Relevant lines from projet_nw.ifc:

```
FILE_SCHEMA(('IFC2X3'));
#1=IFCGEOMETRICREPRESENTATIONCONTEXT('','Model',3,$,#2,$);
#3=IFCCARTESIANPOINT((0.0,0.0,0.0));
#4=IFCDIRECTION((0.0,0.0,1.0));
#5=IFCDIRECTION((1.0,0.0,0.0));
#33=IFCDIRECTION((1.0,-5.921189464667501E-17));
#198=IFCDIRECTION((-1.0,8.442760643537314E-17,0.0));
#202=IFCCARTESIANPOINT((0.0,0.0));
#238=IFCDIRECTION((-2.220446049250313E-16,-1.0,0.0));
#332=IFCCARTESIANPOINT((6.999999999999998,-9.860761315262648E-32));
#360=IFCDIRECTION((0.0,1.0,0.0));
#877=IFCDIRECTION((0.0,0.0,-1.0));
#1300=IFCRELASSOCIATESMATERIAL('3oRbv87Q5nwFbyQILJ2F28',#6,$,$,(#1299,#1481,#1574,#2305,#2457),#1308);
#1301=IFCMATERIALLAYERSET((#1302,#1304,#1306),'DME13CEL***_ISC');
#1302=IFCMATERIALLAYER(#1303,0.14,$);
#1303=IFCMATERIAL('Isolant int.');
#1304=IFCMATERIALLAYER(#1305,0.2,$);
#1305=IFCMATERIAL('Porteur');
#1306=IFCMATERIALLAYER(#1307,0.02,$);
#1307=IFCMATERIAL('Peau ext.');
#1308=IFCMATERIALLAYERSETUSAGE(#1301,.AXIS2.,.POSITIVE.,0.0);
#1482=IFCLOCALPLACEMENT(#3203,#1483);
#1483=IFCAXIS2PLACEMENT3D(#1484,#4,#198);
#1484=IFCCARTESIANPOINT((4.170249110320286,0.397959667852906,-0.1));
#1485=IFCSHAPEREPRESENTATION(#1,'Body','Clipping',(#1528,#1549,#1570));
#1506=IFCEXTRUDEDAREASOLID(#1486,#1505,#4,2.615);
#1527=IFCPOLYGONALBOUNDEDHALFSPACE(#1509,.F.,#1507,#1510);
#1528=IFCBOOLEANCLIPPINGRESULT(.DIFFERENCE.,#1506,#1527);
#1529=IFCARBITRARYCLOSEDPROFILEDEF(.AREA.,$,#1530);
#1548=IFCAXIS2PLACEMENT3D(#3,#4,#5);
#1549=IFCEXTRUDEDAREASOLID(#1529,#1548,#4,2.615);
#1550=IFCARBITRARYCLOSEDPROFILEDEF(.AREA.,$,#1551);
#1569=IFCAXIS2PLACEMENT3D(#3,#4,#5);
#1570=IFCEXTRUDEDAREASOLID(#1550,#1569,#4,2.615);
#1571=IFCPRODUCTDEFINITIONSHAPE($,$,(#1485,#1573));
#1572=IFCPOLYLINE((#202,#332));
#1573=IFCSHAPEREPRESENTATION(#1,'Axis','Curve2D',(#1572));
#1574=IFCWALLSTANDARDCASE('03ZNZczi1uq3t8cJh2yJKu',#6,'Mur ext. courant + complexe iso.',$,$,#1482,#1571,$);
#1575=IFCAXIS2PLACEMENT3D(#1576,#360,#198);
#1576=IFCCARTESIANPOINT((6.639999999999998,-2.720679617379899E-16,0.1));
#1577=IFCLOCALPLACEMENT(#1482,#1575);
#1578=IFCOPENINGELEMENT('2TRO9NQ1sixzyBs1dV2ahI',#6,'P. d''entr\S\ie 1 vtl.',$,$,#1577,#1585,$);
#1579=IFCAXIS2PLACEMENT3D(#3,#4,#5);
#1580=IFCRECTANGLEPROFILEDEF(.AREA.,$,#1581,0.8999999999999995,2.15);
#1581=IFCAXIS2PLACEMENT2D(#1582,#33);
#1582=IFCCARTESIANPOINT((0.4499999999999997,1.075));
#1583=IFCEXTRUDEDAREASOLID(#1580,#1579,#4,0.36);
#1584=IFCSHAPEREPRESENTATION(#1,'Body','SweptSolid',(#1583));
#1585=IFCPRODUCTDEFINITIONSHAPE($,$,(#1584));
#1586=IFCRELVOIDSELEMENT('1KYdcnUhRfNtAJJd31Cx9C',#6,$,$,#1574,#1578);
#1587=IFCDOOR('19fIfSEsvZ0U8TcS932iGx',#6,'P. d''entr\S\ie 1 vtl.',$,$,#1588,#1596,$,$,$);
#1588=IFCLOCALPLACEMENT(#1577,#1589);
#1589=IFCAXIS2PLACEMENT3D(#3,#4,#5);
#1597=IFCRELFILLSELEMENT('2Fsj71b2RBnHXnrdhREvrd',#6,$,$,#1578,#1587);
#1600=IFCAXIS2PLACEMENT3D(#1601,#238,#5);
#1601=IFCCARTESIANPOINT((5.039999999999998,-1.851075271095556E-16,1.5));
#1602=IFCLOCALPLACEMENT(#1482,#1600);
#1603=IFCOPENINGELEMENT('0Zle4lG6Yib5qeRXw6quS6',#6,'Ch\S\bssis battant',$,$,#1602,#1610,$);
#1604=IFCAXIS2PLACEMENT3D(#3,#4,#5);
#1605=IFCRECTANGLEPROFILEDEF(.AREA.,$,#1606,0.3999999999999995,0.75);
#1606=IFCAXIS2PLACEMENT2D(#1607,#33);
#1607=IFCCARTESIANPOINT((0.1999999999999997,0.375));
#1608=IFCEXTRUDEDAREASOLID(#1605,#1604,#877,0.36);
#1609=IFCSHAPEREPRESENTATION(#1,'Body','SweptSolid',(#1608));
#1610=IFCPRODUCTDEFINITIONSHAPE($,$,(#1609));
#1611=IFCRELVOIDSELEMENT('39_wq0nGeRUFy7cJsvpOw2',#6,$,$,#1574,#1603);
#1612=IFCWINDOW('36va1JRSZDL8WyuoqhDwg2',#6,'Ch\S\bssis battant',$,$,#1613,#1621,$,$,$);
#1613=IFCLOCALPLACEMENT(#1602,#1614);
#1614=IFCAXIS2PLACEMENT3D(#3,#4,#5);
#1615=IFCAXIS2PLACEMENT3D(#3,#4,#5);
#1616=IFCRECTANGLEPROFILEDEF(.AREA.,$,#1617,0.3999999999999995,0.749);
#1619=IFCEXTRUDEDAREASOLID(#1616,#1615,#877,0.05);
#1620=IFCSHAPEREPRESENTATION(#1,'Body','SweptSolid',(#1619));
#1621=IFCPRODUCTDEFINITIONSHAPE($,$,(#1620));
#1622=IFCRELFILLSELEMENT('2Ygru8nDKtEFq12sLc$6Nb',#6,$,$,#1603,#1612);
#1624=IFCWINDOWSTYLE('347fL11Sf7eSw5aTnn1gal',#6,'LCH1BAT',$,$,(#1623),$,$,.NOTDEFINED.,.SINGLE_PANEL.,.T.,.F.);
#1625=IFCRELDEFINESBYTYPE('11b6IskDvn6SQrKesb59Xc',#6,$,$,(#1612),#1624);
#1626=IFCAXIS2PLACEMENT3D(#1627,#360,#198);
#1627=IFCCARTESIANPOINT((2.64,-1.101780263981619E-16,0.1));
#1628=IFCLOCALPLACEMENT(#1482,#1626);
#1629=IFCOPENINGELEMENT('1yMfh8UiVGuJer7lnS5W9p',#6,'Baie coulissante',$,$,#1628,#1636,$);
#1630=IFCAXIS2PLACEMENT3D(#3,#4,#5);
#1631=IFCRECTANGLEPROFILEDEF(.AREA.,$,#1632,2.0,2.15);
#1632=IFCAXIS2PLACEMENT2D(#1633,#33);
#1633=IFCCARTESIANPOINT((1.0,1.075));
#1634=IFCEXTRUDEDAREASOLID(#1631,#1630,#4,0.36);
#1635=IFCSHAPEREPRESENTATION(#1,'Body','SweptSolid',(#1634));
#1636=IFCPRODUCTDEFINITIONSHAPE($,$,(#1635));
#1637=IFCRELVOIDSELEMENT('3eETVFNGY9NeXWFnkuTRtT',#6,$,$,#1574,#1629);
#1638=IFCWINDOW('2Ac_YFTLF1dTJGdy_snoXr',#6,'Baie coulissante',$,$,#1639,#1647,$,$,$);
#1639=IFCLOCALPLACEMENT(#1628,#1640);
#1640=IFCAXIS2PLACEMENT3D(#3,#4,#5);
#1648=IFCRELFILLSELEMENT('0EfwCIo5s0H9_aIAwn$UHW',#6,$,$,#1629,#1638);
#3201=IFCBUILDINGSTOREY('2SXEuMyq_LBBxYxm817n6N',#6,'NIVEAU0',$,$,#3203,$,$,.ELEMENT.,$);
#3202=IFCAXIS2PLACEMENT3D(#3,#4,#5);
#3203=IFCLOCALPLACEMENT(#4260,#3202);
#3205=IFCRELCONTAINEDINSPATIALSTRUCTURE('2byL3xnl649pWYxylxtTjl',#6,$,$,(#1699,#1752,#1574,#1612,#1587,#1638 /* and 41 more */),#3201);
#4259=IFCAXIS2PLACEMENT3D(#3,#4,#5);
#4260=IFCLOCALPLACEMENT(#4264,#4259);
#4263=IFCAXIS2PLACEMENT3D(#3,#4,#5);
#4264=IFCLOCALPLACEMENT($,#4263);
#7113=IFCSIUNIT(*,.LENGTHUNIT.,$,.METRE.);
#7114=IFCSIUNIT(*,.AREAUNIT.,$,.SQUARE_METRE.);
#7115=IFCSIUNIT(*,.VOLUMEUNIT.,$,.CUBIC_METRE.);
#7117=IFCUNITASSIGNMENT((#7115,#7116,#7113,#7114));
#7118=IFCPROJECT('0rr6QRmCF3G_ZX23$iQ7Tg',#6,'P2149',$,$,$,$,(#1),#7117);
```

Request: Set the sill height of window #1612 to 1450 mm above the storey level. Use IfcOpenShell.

```python
import numpy as np
import ifcopenshell
import ifcopenshell.api.geometry
import ifcopenshell.geom
import ifcopenshell.util.element
import ifcopenshell.util.placement
import ifcopenshell.util.shape
import ifcopenshell.util.unit

model = ifcopenshell.open("projet_nw.ifc")
unit_scale = ifcopenshell.util.unit.calculate_unit_scale(model)

window = model.by_guid("36va1JRSZDL8WyuoqhDwg2")
opening = window.FillsVoids[0].RelatingOpeningElement
storey = ifcopenshell.util.element.get_container(window, ifc_class="IfcBuildingStorey")
level = ifcopenshell.util.placement.get_local_placement(storey.ObjectPlacement)[2, 3]

# The opening's origin need not be at the sill, so measure its lowest point.
shape = ifcopenshell.geom.create_shape(ifcopenshell.geom.settings(), opening)
bottom = ifcopenshell.util.shape.get_shape_bottom_elevation(shape, shape.geometry) / unit_scale
dz = level + 1.45 / unit_scale - bottom

shift = np.array([0.0, 0.0, dz])
# The window is placed relative to its opening, so it follows when the opening moves.
matrix = ifcopenshell.util.placement.get_local_placement(opening.ObjectPlacement)
matrix[:3, 3] += shift
ifcopenshell.api.geometry.edit_object_placement(
    model, product=opening, matrix=matrix, is_si=False, should_transform_children=True
)

print(f"moved by {dz * unit_scale:+.3f} m")

model.write("projet_nw_rev.ifc")
```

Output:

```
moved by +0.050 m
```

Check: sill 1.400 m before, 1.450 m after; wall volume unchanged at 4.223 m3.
